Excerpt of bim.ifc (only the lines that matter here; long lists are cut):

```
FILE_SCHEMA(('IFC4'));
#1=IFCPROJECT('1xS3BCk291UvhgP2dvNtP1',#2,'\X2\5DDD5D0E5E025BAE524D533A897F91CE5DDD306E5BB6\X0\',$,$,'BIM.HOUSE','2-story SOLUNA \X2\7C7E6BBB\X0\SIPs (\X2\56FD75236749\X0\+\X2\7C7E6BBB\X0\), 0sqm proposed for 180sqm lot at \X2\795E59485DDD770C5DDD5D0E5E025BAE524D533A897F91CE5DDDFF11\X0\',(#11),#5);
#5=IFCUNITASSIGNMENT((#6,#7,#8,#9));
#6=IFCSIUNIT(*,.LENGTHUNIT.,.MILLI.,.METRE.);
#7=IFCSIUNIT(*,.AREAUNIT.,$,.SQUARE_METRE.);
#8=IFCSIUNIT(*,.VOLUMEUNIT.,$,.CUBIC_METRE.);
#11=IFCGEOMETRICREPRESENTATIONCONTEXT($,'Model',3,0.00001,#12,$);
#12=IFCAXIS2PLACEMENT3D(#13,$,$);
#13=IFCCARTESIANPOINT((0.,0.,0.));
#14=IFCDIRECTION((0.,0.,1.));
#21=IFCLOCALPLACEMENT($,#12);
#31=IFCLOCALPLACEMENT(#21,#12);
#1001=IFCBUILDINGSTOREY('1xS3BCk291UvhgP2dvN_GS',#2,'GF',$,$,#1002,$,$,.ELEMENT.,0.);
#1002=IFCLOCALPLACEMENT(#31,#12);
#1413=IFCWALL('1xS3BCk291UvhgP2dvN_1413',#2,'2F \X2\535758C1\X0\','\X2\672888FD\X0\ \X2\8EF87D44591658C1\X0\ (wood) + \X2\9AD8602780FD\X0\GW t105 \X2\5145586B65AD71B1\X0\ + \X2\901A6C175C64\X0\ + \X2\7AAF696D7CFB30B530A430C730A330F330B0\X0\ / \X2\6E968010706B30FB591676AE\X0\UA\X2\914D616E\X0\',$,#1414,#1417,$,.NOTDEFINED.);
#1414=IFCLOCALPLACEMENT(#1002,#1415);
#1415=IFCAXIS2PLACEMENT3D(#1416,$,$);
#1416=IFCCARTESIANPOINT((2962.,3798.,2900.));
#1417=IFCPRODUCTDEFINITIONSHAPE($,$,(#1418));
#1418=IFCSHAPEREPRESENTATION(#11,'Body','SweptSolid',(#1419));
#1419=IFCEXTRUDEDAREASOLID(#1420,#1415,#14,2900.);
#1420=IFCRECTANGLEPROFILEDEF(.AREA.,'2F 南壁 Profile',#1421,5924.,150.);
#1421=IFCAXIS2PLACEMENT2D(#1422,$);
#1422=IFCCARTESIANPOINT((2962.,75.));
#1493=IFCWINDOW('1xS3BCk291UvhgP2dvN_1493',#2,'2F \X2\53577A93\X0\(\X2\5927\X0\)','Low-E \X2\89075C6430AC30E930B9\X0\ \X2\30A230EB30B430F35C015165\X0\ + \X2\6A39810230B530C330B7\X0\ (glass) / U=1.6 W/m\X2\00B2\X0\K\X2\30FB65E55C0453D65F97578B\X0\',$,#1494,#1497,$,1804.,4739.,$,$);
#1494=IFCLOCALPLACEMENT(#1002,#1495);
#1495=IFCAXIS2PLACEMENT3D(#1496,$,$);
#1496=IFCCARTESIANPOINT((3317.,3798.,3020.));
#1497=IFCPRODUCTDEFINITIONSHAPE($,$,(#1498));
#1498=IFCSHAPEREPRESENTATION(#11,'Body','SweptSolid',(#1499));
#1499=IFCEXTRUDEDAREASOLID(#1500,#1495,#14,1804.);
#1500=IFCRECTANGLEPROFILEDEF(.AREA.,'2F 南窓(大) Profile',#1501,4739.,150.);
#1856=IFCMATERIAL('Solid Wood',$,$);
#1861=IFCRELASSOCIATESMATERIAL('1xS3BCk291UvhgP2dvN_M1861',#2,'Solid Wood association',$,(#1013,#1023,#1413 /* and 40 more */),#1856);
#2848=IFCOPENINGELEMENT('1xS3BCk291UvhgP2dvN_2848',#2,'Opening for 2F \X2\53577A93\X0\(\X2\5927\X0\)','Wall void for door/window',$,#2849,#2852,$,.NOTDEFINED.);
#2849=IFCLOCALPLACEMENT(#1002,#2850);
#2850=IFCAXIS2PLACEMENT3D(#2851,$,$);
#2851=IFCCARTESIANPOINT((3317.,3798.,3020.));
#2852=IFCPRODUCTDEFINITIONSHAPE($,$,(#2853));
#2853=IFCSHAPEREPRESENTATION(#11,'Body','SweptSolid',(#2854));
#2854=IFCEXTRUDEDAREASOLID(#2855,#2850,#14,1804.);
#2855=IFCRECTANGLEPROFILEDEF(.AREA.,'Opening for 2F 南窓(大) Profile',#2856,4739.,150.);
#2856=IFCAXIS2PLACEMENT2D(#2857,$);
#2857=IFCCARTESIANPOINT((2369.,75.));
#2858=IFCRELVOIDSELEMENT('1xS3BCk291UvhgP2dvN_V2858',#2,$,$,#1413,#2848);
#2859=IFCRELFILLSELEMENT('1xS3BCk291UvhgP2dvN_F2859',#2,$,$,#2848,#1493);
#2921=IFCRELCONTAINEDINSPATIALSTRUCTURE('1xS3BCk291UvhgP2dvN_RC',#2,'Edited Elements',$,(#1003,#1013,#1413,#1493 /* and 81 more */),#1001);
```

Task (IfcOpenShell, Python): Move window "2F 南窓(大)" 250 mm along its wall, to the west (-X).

```python
import ifcopenshell
import ifcopenshell.api.geometry
import ifcopenshell.util.placement
import ifcopenshell.util.unit

model = ifcopenshell.open("bim.ifc")
unit_scale = ifcopenshell.util.unit.calculate_unit_scale(model)

window = model.by_id(1493)
opening = window.FillsVoids[0].RelatingOpeningElement
wall = opening.VoidsElements[0].RelatingBuildingElement

wall_matrix = ifcopenshell.util.placement.get_local_placement(wall.ObjectPlacement)
shift = wall_matrix[:3, 0] * -0.25 / unit_scale
before = ifcopenshell.util.placement.get_local_placement(window.ObjectPlacement)[:3, 3].copy()

# The window is not placed relative to its opening, so move both.
for product in (opening, window):
    matrix = ifcopenshell.util.placement.get_local_placement(product.ObjectPlacement)
    matrix[:3, 3] += shift
    ifcopenshell.api.geometry.edit_object_placement(model, product=product, matrix=matrix, is_si=False)

after = ifcopenshell.util.placement.get_local_placement(window.ObjectPlacement)[:3, 3]
print("window moved by", (after - before).round(3) + 0.0)

model.write("bim_v2.ifc")
```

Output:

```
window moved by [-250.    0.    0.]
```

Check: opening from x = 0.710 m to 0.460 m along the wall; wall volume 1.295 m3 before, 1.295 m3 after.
